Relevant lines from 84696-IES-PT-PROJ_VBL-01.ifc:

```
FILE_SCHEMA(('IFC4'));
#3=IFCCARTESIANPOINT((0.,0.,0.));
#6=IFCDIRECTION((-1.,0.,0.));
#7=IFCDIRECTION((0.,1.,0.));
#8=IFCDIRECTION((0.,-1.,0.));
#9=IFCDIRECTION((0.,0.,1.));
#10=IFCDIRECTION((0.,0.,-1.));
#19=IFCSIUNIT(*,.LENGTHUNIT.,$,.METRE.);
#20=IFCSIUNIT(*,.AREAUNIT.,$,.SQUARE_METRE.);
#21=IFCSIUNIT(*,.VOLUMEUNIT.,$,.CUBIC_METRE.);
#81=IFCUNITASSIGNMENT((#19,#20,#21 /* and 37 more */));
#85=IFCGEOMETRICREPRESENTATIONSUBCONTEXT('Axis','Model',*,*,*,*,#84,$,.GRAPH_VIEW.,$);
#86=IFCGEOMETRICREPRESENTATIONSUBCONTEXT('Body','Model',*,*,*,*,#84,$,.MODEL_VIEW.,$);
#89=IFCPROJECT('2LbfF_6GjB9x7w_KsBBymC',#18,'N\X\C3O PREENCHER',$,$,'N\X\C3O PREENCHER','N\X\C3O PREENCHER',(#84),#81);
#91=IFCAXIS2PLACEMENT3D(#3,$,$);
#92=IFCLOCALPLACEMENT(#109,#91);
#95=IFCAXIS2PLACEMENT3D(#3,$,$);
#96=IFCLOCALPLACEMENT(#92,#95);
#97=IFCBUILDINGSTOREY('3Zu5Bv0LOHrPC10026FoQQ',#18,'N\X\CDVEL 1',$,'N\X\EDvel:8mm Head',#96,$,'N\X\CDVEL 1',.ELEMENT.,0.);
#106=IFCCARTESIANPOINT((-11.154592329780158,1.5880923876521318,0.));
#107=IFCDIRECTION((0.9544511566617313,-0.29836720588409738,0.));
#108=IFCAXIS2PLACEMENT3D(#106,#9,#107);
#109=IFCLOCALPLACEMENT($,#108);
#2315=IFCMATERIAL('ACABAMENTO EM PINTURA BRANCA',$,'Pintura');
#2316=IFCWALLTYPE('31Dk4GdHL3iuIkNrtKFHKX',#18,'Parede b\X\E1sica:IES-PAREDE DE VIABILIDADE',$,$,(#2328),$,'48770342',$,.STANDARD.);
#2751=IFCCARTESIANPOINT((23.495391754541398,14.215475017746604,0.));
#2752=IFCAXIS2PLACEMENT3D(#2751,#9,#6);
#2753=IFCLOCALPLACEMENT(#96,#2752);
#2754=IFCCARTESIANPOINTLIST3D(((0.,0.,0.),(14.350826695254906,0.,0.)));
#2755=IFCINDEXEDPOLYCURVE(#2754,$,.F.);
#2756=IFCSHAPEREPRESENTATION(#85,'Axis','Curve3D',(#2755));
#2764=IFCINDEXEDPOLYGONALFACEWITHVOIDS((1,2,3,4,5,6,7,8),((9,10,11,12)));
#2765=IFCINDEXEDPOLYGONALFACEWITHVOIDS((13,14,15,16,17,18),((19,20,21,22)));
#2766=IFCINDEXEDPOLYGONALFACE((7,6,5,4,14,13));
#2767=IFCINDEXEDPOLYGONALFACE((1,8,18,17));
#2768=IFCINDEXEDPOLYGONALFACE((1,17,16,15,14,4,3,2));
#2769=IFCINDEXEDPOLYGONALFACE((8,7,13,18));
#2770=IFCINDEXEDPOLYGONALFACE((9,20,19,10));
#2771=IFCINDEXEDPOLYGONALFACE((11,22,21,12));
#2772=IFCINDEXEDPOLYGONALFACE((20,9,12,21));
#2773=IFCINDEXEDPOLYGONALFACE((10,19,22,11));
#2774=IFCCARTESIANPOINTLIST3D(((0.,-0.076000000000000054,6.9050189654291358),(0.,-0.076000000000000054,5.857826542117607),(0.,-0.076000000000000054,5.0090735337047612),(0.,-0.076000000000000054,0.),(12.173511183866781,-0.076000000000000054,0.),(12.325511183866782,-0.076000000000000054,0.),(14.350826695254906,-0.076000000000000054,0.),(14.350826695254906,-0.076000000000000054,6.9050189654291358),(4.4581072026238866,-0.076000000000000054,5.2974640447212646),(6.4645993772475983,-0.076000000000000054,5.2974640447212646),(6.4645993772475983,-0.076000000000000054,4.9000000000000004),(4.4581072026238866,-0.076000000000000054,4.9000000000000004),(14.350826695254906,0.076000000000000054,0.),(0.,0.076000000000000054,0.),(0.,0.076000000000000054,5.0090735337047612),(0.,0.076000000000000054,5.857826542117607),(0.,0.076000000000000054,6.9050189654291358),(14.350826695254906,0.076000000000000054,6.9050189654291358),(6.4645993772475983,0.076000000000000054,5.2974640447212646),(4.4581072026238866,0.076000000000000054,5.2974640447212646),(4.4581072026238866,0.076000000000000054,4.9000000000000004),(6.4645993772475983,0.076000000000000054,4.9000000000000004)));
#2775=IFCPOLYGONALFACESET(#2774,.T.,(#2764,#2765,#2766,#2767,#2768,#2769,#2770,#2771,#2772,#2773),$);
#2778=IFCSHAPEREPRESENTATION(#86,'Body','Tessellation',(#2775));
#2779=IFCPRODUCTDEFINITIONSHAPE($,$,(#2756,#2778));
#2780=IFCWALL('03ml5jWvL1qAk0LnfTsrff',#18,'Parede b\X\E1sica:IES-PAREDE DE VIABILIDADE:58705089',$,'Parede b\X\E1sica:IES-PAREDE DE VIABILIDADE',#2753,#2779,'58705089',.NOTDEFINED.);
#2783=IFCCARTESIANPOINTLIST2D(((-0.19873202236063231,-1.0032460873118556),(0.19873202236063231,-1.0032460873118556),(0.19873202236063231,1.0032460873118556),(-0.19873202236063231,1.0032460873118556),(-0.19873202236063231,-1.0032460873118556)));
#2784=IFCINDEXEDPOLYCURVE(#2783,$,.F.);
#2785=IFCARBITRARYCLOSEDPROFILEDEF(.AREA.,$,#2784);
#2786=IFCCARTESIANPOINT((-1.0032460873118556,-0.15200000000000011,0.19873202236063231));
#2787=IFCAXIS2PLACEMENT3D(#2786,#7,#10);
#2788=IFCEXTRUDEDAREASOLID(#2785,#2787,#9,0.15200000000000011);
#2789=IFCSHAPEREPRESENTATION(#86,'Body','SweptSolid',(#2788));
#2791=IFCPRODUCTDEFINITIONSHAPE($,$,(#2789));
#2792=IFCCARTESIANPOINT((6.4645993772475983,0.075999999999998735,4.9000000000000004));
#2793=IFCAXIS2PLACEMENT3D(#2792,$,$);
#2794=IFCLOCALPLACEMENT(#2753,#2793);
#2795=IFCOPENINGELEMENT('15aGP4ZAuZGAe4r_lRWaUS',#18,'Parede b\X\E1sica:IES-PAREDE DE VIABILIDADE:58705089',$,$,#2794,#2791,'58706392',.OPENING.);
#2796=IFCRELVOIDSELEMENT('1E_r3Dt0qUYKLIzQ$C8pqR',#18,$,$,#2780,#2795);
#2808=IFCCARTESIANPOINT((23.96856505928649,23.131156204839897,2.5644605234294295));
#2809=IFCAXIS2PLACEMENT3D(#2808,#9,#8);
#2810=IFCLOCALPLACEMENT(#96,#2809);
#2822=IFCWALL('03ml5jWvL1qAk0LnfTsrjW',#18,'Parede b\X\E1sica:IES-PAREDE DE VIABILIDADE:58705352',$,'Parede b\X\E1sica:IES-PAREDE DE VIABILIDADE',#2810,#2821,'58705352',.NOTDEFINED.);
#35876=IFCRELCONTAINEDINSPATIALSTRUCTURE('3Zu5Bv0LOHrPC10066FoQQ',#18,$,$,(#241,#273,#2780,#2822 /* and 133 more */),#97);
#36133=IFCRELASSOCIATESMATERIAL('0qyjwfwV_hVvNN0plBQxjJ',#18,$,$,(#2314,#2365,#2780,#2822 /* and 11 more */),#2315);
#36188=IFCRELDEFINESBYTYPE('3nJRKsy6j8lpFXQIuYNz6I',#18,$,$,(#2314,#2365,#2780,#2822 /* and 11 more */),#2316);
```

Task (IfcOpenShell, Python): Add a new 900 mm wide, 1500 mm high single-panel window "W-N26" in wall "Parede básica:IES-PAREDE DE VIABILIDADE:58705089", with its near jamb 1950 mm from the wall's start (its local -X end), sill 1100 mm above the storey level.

```python
import numpy as np
import ifcopenshell
import ifcopenshell.api.feature
import ifcopenshell.api.geometry
import ifcopenshell.api.root
import ifcopenshell.api.spatial
import ifcopenshell.geom
import ifcopenshell.util.element
import ifcopenshell.util.placement
import ifcopenshell.util.representation
import ifcopenshell.util.shape
import ifcopenshell.util.unit

model = ifcopenshell.open("84696-IES-PT-PROJ_VBL-01.ifc")
unit_scale = ifcopenshell.util.unit.calculate_unit_scale(model)
settings = ifcopenshell.geom.settings()


def volume(element):
    """Net volume in cubic metres, openings subtracted."""
    shape = ifcopenshell.geom.create_shape(settings, element)
    return ifcopenshell.util.shape.get_volume(shape.geometry)


wall = model.by_guid("03ml5jWvL1qAk0LnfTsrff")
storey = ifcopenshell.util.element.get_container(wall, ifc_class="IfcBuildingStorey")
context = ifcopenshell.util.representation.get_context(model, "Model", "Body", "MODEL_VIEW")
before = volume(wall)

width, height, from_end, sill = 0.9, 1.5, 1.95, 1.1  # metres

# The wall runs along its own X axis, and the end named is its -X end.
wall_shape = ifcopenshell.geom.create_shape(settings, wall)
x, y, z = ifcopenshell.util.shape.get_vertices(wall_shape.geometry).T
start = x.min() + from_end
face, thickness = float(y.min()), float(y.max() - y.min())
wall_matrix = ifcopenshell.util.placement.get_local_placement(wall.ObjectPlacement)
level = ifcopenshell.util.placement.get_local_placement(storey.ObjectPlacement)[2, 3]


def in_wall(x, y):
    """Placement at x, y metres in the wall's axes, at sill height."""
    matrix = wall_matrix.copy()
    matrix[:, 3] = wall_matrix @ np.array([x / unit_scale, y / unit_scale, 0.0, 1.0])
    matrix[2, 3] = level + sill / unit_scale
    return matrix


# Opening: a box that overshoots both wall faces by 50 mm.
opening = ifcopenshell.api.root.create_entity(model, ifc_class="IfcOpeningElement", predefined_type="OPENING")
box = ifcopenshell.api.geometry.add_wall_representation(
    model, context=context, length=width, height=height, thickness=thickness + 0.1
)
ifcopenshell.api.geometry.assign_representation(model, product=opening, representation=box)
ifcopenshell.api.geometry.edit_object_placement(model, product=opening, matrix=in_wall(start, face - 0.05), is_si=False)
ifcopenshell.api.feature.add_feature(model, feature=opening, element=wall)

window = ifcopenshell.api.root.create_entity(model, ifc_class="IfcWindow", name="W-N26", predefined_type="WINDOW")
window.OverallWidth, window.OverallHeight = width / unit_scale, height / unit_scale
window.PartitioningType = "SINGLE_PANEL"
body = ifcopenshell.api.geometry.add_window_representation(
    model,
    context=context,
    overall_width=window.OverallWidth,
    overall_height=window.OverallHeight,
    partition_type="SINGLE_PANEL",
)
ifcopenshell.api.geometry.assign_representation(model, product=window, representation=body)
ifcopenshell.api.spatial.assign_container(model, products=[window], relating_structure=storey)
ifcopenshell.api.feature.add_filling(model, opening=opening, element=window)

# Centre the window in the wall's thickness.
ifcopenshell.api.geometry.edit_object_placement(model, product=window, matrix=in_wall(start, face), is_si=False)
window_shape = ifcopenshell.geom.create_shape(settings, window)
depth = ifcopenshell.util.shape.get_vertices(window_shape.geometry)[:, 1]
offset = face + thickness / 2 - (depth.min() + depth.max()) / 2
ifcopenshell.api.geometry.edit_object_placement(model, product=window, matrix=in_wall(start, offset), is_si=False)

after = volume(wall)

print(f"wall volume {before:.3f} -> {after:.3f} m3")

model.write("84696-IES-PT-PROJ_VBL-01-out.ifc")
```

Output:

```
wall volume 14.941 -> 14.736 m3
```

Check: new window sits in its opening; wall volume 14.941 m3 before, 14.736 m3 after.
